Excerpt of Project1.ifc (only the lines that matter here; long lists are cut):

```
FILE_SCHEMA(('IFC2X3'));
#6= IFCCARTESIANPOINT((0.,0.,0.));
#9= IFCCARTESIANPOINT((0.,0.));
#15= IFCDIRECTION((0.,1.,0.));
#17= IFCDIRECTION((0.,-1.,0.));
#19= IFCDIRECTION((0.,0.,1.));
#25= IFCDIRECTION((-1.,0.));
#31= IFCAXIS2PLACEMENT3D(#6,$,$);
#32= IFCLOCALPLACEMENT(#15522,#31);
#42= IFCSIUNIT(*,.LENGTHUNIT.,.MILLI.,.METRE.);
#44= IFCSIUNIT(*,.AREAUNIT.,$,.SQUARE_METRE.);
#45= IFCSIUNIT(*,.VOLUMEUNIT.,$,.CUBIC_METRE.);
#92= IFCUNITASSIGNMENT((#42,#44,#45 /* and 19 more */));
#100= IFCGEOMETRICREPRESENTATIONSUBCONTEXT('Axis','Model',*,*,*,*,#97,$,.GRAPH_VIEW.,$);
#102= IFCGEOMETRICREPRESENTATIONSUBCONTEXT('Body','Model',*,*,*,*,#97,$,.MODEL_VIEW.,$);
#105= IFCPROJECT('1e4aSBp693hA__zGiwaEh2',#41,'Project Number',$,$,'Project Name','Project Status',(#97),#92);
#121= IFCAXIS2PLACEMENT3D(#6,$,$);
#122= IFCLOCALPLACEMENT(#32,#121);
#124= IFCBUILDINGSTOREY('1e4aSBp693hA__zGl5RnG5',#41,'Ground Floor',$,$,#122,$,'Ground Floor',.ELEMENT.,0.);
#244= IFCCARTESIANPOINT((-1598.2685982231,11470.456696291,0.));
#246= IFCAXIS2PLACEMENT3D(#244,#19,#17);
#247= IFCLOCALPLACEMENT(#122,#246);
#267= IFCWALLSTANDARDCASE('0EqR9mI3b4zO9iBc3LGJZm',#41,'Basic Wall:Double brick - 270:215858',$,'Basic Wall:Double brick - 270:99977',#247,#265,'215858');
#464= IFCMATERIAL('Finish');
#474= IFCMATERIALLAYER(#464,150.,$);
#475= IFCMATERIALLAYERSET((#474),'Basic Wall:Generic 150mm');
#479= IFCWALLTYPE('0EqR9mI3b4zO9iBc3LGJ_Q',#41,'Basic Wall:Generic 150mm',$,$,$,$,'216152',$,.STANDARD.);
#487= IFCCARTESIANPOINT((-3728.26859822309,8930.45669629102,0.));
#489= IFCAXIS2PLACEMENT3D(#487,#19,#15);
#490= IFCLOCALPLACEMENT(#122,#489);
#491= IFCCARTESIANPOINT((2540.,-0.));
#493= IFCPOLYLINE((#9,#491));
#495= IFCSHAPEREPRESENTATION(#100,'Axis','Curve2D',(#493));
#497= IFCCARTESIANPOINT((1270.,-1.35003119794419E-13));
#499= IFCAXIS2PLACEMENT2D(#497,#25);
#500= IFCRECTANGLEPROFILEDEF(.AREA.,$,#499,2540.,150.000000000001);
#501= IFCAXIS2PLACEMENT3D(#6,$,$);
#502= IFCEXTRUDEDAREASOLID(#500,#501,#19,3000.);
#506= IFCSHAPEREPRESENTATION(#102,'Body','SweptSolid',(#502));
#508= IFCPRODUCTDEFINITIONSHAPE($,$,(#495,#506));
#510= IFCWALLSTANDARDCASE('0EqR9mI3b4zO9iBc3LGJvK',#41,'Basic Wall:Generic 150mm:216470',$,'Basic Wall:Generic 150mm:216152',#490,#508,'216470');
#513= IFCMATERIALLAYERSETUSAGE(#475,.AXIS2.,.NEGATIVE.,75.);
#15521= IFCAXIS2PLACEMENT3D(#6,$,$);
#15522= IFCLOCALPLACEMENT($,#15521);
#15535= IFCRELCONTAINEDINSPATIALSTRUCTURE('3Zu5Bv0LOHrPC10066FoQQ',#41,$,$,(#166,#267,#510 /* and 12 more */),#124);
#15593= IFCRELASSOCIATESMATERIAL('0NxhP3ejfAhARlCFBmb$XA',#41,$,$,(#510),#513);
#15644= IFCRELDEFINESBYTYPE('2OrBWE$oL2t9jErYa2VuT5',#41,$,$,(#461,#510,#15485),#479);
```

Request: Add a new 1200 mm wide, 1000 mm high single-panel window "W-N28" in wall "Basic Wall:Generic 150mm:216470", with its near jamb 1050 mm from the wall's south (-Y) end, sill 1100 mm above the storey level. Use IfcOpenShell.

```python
import numpy as np
import ifcopenshell
import ifcopenshell.api.feature
import ifcopenshell.api.geometry
import ifcopenshell.api.root
import ifcopenshell.api.spatial
import ifcopenshell.api.type
import ifcopenshell.geom
import ifcopenshell.util.element
import ifcopenshell.util.placement
import ifcopenshell.util.representation
import ifcopenshell.util.shape
import ifcopenshell.util.unit

model = ifcopenshell.open("Project1.ifc")
unit_scale = ifcopenshell.util.unit.calculate_unit_scale(model)
settings = ifcopenshell.geom.settings()


def volume(element):
    """Net volume in cubic metres, openings subtracted."""
    shape = ifcopenshell.geom.create_shape(settings, element)
    return ifcopenshell.util.shape.get_volume(shape.geometry)


wall = model.by_guid("0EqR9mI3b4zO9iBc3LGJvK")
storey = ifcopenshell.util.element.get_container(wall, ifc_class="IfcBuildingStorey")
context = ifcopenshell.util.representation.get_context(model, "Model", "Body", "MODEL_VIEW")
before = volume(wall)

width, height, from_end, sill = 1.2, 1, 1.05, 1.1  # metres

# The wall runs along its own X axis, and the end named is its -X end.
wall_shape = ifcopenshell.geom.create_shape(settings, wall)
x, y, z = ifcopenshell.util.shape.get_vertices(wall_shape.geometry).T
start = x.min() + from_end
face, thickness = float(y.min()), float(y.max() - y.min())
wall_matrix = ifcopenshell.util.placement.get_local_placement(wall.ObjectPlacement)
level = ifcopenshell.util.placement.get_local_placement(storey.ObjectPlacement)[2, 3]


def in_wall(x, y):
    """Placement at x, y metres in the wall's axes, at sill height."""
    matrix = wall_matrix.copy()
    matrix[:, 3] = wall_matrix @ np.array([x / unit_scale, y / unit_scale, 0.0, 1.0])
    matrix[2, 3] = level + sill / unit_scale
    return matrix


# Opening: a box that overshoots both wall faces by 50 mm.
opening = ifcopenshell.api.root.create_entity(model, ifc_class="IfcOpeningElement")
box = ifcopenshell.api.geometry.add_wall_representation(
    model, context=context, length=width, height=height, thickness=thickness + 0.1
)
ifcopenshell.api.geometry.assign_representation(model, product=opening, representation=box)
ifcopenshell.api.geometry.edit_object_placement(model, product=opening, matrix=in_wall(start, face - 0.05), is_si=False)
ifcopenshell.api.feature.add_feature(model, feature=opening, element=wall)

window = ifcopenshell.api.root.create_entity(model, ifc_class="IfcWindow", name="W-N28")
window.OverallWidth, window.OverallHeight = width / unit_scale, height / unit_scale
body = ifcopenshell.api.geometry.add_window_representation(
    model,
    context=context,
    overall_width=window.OverallWidth,
    overall_height=window.OverallHeight,
    partition_type="SINGLE_PANEL",
)
ifcopenshell.api.geometry.assign_representation(model, product=window, representation=body)
ifcopenshell.api.spatial.assign_container(model, products=[window], relating_structure=storey)
fills = ifcopenshell.api.feature.add_filling(model, opening=opening, element=window)
fills.OwnerHistory = window.OwnerHistory  # required in IFC2X3

# IFC2X3 keeps the operation on the window style.
style = ifcopenshell.api.root.create_entity(model, ifc_class="IfcWindowStyle", name="W-N28")
style.OperationType, style.ConstructionType = "SINGLE_PANEL", "NOTDEFINED"
style.ParameterTakesPrecedence = style.Sizeable = False
ifcopenshell.api.type.assign_type(model, related_objects=[window], relating_type=style)

# Centre the window in the wall's thickness.
ifcopenshell.api.geometry.edit_object_placement(model, product=window, matrix=in_wall(start, face), is_si=False)
window_shape = ifcopenshell.geom.create_shape(settings, window)
depth = ifcopenshell.util.shape.get_vertices(window_shape.geometry)[:, 1]
offset = face + thickness / 2 - (depth.min() + depth.max()) / 2
ifcopenshell.api.geometry.edit_object_placement(model, product=window, matrix=in_wall(start, offset), is_si=False)

after = volume(wall)

print(f"wall volume {before:.3f} -> {after:.3f} m3")

model.write("Project1_edited.ifc")
```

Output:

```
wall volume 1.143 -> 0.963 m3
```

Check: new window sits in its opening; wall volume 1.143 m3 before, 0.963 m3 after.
